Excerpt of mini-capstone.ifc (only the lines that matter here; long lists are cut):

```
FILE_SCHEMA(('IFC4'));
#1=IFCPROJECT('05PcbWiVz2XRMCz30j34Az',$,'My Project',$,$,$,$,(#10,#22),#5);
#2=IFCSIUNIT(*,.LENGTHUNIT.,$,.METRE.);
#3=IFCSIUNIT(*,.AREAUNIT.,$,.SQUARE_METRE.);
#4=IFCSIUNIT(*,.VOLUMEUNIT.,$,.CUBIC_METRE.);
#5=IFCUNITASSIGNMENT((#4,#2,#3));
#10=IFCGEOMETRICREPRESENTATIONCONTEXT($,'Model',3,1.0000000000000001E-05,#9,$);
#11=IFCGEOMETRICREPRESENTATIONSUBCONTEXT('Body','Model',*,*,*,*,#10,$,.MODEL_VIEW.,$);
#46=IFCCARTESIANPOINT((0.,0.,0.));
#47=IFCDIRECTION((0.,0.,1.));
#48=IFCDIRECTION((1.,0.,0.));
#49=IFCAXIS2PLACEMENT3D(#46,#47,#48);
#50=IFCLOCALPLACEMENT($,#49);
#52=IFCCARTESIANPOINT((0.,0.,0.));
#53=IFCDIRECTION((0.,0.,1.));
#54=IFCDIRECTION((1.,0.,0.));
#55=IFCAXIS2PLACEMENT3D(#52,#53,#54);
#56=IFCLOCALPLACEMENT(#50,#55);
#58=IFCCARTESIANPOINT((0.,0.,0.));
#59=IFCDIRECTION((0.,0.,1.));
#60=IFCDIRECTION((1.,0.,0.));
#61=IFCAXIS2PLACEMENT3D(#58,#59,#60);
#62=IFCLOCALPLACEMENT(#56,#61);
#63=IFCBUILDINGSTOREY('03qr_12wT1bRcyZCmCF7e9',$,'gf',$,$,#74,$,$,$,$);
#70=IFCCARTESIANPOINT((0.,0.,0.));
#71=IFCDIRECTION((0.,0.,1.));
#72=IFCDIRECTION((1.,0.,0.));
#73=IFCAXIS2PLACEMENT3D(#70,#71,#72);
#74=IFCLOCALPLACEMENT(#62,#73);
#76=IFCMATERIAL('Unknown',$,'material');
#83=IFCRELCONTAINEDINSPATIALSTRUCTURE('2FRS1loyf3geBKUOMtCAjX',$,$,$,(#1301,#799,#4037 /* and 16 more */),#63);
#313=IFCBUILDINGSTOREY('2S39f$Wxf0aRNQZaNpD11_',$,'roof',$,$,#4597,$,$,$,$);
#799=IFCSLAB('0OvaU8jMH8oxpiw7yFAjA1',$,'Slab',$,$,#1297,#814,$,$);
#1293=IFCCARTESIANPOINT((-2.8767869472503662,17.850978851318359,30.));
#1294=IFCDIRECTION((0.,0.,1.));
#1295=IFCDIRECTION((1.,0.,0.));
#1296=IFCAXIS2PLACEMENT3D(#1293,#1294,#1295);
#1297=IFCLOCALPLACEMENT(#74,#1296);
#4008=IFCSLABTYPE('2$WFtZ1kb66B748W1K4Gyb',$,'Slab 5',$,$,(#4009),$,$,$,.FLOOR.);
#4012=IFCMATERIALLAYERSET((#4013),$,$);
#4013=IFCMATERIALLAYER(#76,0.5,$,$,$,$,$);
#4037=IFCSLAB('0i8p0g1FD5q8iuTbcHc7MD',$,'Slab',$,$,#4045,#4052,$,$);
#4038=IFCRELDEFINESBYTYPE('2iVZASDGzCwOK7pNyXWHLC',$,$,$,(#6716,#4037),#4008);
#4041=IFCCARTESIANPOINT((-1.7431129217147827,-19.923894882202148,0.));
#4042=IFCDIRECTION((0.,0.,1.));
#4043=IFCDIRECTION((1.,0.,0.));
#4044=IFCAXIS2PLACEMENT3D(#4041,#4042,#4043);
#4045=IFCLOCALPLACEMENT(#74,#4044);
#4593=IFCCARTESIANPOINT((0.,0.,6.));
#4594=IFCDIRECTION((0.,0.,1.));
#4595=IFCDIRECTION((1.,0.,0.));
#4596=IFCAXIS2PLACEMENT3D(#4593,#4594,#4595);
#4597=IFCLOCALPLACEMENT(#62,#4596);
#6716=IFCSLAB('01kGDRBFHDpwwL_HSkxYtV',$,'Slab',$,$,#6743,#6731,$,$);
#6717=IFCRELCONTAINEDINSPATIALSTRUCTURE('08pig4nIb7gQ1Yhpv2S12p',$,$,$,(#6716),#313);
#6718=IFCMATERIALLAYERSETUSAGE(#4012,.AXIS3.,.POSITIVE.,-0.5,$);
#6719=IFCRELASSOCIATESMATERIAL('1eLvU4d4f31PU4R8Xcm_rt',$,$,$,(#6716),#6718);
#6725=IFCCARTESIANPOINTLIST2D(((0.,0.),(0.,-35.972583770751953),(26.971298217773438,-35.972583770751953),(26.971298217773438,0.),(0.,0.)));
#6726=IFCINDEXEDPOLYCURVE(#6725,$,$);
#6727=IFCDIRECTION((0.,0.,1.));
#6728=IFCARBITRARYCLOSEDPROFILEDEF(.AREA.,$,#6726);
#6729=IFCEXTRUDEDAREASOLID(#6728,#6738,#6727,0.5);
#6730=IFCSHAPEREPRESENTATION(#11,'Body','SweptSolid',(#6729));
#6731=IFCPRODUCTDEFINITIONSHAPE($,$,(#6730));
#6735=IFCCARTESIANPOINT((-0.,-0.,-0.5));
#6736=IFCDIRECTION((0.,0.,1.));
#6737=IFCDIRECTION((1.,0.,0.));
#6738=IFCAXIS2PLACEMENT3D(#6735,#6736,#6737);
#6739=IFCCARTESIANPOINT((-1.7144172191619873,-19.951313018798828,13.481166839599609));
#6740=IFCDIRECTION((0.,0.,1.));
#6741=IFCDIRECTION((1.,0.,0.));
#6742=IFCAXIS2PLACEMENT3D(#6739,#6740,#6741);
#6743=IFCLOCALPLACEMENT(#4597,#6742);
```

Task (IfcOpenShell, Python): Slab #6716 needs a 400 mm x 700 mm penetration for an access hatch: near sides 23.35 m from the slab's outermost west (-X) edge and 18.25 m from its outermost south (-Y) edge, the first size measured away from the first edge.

```python
import numpy as np
import ifcopenshell
import ifcopenshell.api.feature
import ifcopenshell.api.geometry
import ifcopenshell.api.root
import ifcopenshell.geom
import ifcopenshell.util.placement
import ifcopenshell.util.representation
import ifcopenshell.util.shape
import ifcopenshell.util.unit

model = ifcopenshell.open("mini-capstone.ifc")
unit_scale = ifcopenshell.util.unit.calculate_unit_scale(model)
settings = ifcopenshell.geom.settings()


def volume(element):
    """Net volume in cubic metres, openings subtracted."""
    shape = ifcopenshell.geom.create_shape(settings, element)
    return ifcopenshell.util.shape.get_volume(shape.geometry)


slab = model.by_guid("01kGDRBFHDpwwL_HSkxYtV")
before = volume(slab)

# Extent in the slab's own axes, in metres. The edges named are its -X and -Y sides.
slab_shape = ifcopenshell.geom.create_shape(settings, slab)
vertices = ifcopenshell.util.shape.get_vertices(slab_shape.geometry)
x_min, y_min, bottom = vertices.min(axis=0)
top = vertices[:, 2].max()

opening = ifcopenshell.api.root.create_entity(model, ifc_class="IfcOpeningElement", name="Access hatch opening", predefined_type="OPENING")
context = ifcopenshell.util.representation.get_context(model, "Model", "Body", "MODEL_VIEW")
width, depth = 0.4, 0.7
outline = [(0.0, 0.0), (width, 0.0), (width, depth), (0.0, depth), (0.0, 0.0)]
# Overshoot both faces by 50 mm so the cut is clean.
shape = ifcopenshell.api.geometry.add_slab_representation(
    model, context=context, depth=top - bottom + 0.1, polyline=outline
)
ifcopenshell.api.geometry.assign_representation(model, product=opening, representation=shape)

matrix = ifcopenshell.util.placement.get_local_placement(slab.ObjectPlacement)
matrix[:, 3] = matrix @ np.append(np.array([x_min + 23.35, y_min + 18.25, bottom - 0.05]) / unit_scale, 1.0)
ifcopenshell.api.geometry.edit_object_placement(model, product=opening, matrix=matrix, is_si=False)
ifcopenshell.api.feature.add_feature(model, feature=opening, element=slab)

after = volume(slab)

print(f"slab volume {before:.3f} -> {after:.3f} m3")

model.write("mini-capstone_updated.ifc")
```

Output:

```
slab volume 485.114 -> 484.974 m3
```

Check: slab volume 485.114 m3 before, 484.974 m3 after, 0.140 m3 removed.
